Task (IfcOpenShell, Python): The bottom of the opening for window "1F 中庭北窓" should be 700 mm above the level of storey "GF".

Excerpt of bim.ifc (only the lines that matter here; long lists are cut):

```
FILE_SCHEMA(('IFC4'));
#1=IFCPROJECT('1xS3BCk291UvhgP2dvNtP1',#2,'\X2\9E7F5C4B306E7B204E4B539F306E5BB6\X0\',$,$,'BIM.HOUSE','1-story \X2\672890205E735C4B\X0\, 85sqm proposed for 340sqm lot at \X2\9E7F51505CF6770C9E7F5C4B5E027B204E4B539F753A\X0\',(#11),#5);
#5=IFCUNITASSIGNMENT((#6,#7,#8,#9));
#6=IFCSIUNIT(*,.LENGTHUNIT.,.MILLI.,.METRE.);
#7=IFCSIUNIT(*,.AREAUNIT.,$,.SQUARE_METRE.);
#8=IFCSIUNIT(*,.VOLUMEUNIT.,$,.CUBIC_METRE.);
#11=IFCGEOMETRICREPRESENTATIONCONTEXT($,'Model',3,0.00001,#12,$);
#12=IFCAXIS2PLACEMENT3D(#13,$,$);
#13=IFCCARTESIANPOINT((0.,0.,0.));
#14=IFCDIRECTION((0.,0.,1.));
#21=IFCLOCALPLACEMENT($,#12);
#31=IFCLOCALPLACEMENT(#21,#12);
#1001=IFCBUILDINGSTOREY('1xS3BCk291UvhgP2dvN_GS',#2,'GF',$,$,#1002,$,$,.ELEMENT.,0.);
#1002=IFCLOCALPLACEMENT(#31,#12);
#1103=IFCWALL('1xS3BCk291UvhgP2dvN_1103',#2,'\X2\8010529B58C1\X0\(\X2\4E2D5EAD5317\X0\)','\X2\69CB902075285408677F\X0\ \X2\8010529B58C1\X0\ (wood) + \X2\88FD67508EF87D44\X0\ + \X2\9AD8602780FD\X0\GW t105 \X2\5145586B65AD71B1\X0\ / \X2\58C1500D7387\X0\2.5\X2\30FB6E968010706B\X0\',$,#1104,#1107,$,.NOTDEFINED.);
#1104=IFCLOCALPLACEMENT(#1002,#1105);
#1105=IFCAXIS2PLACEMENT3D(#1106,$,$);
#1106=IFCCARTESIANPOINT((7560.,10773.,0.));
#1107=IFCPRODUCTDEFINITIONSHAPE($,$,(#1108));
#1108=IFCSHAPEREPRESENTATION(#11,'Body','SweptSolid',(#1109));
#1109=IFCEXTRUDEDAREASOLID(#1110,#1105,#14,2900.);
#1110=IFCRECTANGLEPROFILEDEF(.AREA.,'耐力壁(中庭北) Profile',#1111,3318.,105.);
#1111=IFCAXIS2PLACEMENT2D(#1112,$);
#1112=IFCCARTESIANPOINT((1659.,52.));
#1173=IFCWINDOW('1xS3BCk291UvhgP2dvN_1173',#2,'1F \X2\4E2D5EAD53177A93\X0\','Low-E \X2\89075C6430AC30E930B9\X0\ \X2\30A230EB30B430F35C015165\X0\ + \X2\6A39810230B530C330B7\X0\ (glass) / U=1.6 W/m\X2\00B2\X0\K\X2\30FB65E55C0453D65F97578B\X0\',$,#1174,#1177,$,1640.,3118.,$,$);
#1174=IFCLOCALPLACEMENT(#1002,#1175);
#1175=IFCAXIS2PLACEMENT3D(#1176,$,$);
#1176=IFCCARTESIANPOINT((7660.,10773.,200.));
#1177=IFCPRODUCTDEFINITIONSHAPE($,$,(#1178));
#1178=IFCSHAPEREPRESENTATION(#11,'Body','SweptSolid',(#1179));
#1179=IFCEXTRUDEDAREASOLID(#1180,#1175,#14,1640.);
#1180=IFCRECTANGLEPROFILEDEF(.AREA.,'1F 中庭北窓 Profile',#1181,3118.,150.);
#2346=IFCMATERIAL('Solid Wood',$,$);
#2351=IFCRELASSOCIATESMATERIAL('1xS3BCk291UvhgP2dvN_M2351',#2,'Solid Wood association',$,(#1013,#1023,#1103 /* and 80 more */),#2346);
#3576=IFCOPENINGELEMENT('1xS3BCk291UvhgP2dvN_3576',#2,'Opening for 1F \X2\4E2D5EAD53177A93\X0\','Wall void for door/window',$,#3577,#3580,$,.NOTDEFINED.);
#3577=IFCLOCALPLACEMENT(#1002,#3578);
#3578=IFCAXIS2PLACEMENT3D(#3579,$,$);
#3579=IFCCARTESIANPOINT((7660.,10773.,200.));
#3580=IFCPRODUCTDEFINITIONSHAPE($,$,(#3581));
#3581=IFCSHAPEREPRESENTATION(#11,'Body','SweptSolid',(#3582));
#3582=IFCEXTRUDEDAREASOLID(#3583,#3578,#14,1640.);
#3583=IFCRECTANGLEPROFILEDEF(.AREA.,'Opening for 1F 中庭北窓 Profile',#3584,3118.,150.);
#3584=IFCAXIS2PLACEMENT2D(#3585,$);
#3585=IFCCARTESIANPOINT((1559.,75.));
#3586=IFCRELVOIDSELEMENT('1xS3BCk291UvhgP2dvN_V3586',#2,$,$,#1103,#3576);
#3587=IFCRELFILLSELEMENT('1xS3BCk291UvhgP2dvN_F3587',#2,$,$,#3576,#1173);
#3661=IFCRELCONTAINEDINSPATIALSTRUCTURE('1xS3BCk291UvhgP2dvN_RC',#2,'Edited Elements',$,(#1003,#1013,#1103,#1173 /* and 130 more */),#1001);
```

```python
import numpy as np
import ifcopenshell
import ifcopenshell.api.geometry
import ifcopenshell.geom
import ifcopenshell.util.element
import ifcopenshell.util.placement
import ifcopenshell.util.shape
import ifcopenshell.util.unit

model = ifcopenshell.open("bim.ifc")
unit_scale = ifcopenshell.util.unit.calculate_unit_scale(model)

window = model.by_id(1173)
opening = window.FillsVoids[0].RelatingOpeningElement
storey = ifcopenshell.util.element.get_container(window, ifc_class="IfcBuildingStorey")
level = ifcopenshell.util.placement.get_local_placement(storey.ObjectPlacement)[2, 3]

# The opening's origin need not be at the sill, so measure its lowest point.
shape = ifcopenshell.geom.create_shape(ifcopenshell.geom.settings(), opening)
bottom = ifcopenshell.util.shape.get_shape_bottom_elevation(shape, shape.geometry) / unit_scale
dz = level + 0.7 / unit_scale - bottom

shift = np.array([0.0, 0.0, dz])
# The window is not placed relative to its opening, so move both.
for product in (opening, window):
    matrix = ifcopenshell.util.placement.get_local_placement(product.ObjectPlacement)
    matrix[:3, 3] += shift
    ifcopenshell.api.geometry.edit_object_placement(model, product=product, matrix=matrix, is_si=False)

print(f"moved by {dz * unit_scale:+.3f} m")

model.write("bim_edited.ifc")
```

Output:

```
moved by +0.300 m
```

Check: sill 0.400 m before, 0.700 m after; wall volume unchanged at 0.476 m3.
